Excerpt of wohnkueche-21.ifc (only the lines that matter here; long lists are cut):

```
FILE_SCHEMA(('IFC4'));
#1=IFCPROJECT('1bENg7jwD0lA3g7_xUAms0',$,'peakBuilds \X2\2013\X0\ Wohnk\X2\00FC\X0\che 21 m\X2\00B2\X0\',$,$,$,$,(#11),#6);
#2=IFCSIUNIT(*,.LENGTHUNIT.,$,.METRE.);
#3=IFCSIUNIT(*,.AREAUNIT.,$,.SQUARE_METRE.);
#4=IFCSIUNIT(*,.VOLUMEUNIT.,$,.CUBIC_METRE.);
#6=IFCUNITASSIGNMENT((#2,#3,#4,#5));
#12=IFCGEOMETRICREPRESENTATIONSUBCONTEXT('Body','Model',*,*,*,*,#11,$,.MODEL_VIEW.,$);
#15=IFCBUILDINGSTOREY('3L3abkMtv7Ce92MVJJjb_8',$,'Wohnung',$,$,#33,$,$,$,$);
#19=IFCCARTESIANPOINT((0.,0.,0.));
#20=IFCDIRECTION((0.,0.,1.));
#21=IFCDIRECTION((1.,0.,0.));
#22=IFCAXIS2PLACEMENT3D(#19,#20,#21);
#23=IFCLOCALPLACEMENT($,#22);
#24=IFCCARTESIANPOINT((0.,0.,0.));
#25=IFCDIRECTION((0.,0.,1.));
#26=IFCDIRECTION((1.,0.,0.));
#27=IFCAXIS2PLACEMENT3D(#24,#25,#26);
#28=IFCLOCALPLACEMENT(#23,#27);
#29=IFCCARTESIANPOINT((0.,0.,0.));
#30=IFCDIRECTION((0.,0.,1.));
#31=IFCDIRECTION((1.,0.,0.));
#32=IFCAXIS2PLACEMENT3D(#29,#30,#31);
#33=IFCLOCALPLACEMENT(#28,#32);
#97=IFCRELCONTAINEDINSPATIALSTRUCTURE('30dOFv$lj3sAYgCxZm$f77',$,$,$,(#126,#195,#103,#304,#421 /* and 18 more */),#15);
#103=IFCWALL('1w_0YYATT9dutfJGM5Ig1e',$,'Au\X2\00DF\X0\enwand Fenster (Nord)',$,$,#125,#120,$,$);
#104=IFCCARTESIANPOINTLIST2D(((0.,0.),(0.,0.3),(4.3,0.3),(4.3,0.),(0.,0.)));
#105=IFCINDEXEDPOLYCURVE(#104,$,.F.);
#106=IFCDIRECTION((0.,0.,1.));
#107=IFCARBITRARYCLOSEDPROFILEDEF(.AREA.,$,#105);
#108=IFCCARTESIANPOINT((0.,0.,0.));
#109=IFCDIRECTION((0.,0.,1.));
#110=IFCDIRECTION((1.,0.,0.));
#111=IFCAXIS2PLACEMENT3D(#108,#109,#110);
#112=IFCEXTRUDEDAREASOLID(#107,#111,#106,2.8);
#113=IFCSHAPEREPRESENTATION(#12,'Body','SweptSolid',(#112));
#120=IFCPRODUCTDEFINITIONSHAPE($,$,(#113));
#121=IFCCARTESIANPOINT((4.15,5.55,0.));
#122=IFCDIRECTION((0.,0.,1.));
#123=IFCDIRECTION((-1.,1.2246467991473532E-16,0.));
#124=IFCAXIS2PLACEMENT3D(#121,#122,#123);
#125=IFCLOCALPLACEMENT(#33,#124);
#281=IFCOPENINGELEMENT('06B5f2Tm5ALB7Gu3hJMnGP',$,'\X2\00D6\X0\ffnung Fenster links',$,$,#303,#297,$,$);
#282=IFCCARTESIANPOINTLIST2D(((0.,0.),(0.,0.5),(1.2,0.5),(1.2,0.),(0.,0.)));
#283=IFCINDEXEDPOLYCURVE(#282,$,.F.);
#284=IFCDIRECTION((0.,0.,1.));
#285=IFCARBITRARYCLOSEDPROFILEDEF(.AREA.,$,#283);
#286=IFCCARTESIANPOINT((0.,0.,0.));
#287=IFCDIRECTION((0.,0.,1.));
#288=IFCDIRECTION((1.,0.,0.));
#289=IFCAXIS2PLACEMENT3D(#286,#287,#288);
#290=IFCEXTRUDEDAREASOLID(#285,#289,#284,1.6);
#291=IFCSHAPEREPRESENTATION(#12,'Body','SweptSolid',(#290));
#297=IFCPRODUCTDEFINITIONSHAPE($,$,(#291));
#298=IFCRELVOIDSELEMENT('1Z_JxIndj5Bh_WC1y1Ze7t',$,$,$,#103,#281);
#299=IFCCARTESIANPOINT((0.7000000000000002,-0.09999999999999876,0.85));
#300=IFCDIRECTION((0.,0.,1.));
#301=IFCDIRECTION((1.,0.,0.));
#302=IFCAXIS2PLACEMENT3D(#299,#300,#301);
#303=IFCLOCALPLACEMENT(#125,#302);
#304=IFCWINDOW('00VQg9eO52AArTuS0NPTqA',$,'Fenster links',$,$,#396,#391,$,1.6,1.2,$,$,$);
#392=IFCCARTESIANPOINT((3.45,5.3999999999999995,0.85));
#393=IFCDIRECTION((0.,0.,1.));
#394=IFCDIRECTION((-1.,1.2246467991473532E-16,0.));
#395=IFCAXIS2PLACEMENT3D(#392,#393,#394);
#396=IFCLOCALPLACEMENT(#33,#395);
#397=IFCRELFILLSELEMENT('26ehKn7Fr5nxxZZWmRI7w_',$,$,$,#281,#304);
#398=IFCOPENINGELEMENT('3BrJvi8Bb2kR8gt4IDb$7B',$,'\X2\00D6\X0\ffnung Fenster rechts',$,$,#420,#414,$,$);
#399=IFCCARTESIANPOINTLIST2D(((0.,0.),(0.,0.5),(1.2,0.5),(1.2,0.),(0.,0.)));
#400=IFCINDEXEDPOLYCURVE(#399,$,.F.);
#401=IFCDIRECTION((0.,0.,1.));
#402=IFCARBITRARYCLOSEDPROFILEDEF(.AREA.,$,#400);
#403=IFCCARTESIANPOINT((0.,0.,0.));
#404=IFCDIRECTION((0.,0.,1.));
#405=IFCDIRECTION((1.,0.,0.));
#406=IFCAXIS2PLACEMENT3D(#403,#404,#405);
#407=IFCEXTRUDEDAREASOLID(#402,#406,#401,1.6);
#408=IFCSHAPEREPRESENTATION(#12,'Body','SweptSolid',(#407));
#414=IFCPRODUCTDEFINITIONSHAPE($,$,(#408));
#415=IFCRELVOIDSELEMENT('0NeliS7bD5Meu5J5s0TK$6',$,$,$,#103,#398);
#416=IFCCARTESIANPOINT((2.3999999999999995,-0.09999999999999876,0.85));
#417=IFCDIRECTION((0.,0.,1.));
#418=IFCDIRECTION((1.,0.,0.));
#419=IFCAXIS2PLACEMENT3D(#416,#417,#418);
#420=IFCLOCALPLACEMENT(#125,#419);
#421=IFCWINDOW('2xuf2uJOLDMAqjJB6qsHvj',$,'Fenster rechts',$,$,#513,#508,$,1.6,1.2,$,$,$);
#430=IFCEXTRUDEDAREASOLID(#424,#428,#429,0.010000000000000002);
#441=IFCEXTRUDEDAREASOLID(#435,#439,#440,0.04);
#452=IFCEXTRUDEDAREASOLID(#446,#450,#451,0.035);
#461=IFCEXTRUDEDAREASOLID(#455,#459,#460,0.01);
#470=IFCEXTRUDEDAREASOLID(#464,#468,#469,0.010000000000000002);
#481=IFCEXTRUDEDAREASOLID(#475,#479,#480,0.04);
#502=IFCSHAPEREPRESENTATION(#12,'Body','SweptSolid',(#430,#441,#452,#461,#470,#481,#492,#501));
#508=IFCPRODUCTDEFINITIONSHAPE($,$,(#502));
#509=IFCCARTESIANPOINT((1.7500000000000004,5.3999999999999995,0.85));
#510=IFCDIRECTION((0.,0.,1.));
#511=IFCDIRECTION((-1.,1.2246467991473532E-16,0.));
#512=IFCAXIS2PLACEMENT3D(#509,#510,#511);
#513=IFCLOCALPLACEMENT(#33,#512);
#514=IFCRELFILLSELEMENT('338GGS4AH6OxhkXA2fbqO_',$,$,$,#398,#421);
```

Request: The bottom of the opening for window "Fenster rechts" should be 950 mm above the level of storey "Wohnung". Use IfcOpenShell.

```python
import numpy as np
import ifcopenshell
import ifcopenshell.api.geometry
import ifcopenshell.geom
import ifcopenshell.util.element
import ifcopenshell.util.placement
import ifcopenshell.util.shape
import ifcopenshell.util.unit

model = ifcopenshell.open("wohnkueche-21.ifc")
unit_scale = ifcopenshell.util.unit.calculate_unit_scale(model)

window = model.by_guid("2xuf2uJOLDMAqjJB6qsHvj")
opening = window.FillsVoids[0].RelatingOpeningElement
storey = ifcopenshell.util.element.get_container(window, ifc_class="IfcBuildingStorey")
level = ifcopenshell.util.placement.get_local_placement(storey.ObjectPlacement)[2, 3]

# The opening's origin need not be at the sill, so measure its lowest point.
shape = ifcopenshell.geom.create_shape(ifcopenshell.geom.settings(), opening)
bottom = ifcopenshell.util.shape.get_shape_bottom_elevation(shape, shape.geometry) / unit_scale
dz = level + 0.95 - bottom

shift = np.array([0.0, 0.0, dz])
# The window is not placed relative to its opening, so move both.
for product in (opening, window):
    matrix = ifcopenshell.util.placement.get_local_placement(product.ObjectPlacement)
    matrix[:3, 3] += shift
    ifcopenshell.api.geometry.edit_object_placement(model, product=product, matrix=matrix, is_si=False)

print(f"moved by {dz * unit_scale:+.3f} m")

model.write("wohnkueche-21-out.ifc")
```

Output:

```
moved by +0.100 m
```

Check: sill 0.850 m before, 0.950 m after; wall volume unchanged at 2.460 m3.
